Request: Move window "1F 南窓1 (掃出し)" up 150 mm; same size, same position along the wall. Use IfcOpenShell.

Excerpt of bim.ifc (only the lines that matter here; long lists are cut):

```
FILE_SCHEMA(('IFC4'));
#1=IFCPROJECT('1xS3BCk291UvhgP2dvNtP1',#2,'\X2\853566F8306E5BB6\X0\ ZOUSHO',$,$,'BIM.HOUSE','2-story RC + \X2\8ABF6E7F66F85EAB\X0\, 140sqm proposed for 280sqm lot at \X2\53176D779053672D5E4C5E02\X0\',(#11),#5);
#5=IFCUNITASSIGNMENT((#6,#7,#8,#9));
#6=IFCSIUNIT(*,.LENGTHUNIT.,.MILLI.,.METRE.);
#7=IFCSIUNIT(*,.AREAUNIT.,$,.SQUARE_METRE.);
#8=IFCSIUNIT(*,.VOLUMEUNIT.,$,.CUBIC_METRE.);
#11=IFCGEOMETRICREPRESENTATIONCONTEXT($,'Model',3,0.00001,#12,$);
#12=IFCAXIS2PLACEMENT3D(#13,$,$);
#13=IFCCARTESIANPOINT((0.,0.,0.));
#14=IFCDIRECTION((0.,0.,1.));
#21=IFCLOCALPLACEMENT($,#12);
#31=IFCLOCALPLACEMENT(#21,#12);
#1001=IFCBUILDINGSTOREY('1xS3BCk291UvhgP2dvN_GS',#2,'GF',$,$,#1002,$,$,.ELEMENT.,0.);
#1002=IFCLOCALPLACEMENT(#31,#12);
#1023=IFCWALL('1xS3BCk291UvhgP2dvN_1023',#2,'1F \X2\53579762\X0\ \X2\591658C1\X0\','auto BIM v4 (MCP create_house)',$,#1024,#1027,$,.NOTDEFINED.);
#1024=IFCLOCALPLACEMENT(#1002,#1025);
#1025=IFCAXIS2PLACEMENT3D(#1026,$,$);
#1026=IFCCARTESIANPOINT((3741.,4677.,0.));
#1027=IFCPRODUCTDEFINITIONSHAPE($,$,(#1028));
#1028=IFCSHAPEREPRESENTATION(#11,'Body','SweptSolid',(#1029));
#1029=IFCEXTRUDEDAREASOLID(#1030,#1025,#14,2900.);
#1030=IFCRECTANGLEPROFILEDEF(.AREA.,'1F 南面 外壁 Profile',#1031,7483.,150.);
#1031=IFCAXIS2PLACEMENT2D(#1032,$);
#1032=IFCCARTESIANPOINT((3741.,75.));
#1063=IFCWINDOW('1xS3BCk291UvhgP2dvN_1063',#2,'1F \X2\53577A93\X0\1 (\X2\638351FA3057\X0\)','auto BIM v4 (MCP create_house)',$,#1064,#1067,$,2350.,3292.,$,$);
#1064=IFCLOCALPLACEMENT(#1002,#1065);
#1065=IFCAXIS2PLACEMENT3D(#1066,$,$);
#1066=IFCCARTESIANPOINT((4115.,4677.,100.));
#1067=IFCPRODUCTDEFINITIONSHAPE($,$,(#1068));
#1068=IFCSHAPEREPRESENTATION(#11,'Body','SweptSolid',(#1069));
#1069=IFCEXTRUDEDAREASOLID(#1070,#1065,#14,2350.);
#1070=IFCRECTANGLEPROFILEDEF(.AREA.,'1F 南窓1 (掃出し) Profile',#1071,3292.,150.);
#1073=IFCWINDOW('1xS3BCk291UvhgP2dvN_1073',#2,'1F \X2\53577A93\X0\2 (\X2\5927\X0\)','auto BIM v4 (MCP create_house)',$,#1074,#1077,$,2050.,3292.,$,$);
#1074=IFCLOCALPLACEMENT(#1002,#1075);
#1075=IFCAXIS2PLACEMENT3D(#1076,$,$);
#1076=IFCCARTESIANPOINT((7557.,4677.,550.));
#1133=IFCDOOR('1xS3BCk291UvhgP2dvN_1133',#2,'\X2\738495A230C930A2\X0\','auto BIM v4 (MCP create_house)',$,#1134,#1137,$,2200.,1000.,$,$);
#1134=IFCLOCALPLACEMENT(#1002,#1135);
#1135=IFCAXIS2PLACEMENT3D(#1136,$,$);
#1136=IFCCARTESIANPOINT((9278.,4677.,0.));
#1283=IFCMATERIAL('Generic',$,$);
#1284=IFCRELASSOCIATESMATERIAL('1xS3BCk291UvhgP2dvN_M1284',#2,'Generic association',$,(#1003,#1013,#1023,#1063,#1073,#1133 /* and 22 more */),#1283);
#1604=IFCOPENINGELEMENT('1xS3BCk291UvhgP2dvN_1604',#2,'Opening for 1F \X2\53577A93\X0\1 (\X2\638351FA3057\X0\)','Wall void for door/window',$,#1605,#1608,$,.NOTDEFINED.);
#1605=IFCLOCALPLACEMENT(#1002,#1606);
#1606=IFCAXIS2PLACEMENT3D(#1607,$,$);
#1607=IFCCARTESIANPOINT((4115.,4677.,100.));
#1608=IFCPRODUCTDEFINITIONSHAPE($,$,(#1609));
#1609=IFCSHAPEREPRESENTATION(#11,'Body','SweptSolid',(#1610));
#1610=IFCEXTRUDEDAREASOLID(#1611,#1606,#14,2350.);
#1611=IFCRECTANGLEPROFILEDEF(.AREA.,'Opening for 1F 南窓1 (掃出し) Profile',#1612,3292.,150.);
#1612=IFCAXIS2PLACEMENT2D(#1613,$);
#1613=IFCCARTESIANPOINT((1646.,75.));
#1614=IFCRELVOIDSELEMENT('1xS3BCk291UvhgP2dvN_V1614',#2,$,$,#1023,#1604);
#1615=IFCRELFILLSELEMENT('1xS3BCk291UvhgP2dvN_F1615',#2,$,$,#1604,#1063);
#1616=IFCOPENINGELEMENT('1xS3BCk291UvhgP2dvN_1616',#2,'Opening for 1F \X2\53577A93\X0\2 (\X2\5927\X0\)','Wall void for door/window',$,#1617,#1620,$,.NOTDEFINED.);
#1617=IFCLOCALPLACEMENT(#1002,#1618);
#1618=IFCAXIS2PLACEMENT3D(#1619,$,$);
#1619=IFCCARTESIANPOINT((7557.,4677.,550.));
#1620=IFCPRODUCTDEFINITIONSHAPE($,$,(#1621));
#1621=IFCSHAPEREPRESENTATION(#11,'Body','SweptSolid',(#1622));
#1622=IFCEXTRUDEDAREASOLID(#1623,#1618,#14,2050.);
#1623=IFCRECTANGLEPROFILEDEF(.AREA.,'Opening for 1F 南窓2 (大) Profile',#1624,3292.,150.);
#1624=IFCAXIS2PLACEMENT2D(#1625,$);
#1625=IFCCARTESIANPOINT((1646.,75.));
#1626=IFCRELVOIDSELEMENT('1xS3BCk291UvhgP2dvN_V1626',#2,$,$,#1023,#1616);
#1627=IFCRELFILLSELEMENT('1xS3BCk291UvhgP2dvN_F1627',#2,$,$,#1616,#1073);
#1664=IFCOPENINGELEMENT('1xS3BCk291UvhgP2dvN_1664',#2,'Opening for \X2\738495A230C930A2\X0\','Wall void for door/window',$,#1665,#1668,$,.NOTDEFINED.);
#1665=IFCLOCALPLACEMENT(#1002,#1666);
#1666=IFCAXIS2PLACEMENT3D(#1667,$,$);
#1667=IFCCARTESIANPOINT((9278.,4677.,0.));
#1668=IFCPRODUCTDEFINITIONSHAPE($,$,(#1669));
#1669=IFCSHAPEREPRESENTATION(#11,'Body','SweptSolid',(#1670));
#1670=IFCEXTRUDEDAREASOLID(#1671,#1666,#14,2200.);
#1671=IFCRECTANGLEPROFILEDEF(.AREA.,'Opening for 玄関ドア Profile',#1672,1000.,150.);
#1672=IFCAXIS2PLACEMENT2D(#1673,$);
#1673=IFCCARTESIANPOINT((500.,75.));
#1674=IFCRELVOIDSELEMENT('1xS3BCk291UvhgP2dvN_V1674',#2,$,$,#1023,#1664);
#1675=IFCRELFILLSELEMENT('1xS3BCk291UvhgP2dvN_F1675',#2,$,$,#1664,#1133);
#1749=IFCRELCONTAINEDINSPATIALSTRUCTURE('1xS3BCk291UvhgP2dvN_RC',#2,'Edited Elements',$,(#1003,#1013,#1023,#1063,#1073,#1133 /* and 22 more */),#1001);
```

```python
import numpy as np
import ifcopenshell
import ifcopenshell.api.geometry
import ifcopenshell.util.placement
import ifcopenshell.util.unit

model = ifcopenshell.open("bim.ifc")
unit_scale = ifcopenshell.util.unit.calculate_unit_scale(model)

window = model.by_guid("1xS3BCk291UvhgP2dvN_1063")
opening = window.FillsVoids[0].RelatingOpeningElement
dz = 150.0

shift = np.array([0.0, 0.0, dz])
# The window is not placed relative to its opening, so move both.
for product in (opening, window):
    matrix = ifcopenshell.util.placement.get_local_placement(product.ObjectPlacement)
    matrix[:3, 3] += shift
    ifcopenshell.api.geometry.edit_object_placement(model, product=product, matrix=matrix, is_si=False)

print(f"moved by {dz * unit_scale:+.3f} m")

model.write("bim_edited.ifc")
```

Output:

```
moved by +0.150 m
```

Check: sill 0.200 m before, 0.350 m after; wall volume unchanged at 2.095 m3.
